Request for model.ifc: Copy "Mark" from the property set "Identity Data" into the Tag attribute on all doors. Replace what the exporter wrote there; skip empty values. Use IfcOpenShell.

First a look at what the model holds.

```python
import ifcopenshell
import ifcopenshell.util.element

model = ifcopenshell.open("model.ifc")
print(model.schema)
doors = model.by_type("IfcDoor")
print(len(doors), "doors")
for e in doors[:8]:
    source = ifcopenshell.util.element.get_pset(e, "Identity Data", "Mark")
    target = e.Tag
    print(e.id(), repr(source), repr(target), sep=" | ")
```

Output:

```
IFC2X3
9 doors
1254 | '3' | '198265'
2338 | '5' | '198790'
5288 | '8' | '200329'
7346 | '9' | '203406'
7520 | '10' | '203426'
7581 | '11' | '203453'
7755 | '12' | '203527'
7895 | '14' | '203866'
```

```python
import ifcopenshell
import ifcopenshell.util.element

model = ifcopenshell.open("model.ifc")

count = 0
for e in model.by_type("IfcDoor"):
    value = ifcopenshell.util.element.get_pset(e, "Identity Data", "Mark")
    current = e.Tag
    if not value or not value.strip() or current == value:
        continue
    e.Tag = value
    count += 1

print(count, "doors updated")

model.write("model_edited.ifc")
```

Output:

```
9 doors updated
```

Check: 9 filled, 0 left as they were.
